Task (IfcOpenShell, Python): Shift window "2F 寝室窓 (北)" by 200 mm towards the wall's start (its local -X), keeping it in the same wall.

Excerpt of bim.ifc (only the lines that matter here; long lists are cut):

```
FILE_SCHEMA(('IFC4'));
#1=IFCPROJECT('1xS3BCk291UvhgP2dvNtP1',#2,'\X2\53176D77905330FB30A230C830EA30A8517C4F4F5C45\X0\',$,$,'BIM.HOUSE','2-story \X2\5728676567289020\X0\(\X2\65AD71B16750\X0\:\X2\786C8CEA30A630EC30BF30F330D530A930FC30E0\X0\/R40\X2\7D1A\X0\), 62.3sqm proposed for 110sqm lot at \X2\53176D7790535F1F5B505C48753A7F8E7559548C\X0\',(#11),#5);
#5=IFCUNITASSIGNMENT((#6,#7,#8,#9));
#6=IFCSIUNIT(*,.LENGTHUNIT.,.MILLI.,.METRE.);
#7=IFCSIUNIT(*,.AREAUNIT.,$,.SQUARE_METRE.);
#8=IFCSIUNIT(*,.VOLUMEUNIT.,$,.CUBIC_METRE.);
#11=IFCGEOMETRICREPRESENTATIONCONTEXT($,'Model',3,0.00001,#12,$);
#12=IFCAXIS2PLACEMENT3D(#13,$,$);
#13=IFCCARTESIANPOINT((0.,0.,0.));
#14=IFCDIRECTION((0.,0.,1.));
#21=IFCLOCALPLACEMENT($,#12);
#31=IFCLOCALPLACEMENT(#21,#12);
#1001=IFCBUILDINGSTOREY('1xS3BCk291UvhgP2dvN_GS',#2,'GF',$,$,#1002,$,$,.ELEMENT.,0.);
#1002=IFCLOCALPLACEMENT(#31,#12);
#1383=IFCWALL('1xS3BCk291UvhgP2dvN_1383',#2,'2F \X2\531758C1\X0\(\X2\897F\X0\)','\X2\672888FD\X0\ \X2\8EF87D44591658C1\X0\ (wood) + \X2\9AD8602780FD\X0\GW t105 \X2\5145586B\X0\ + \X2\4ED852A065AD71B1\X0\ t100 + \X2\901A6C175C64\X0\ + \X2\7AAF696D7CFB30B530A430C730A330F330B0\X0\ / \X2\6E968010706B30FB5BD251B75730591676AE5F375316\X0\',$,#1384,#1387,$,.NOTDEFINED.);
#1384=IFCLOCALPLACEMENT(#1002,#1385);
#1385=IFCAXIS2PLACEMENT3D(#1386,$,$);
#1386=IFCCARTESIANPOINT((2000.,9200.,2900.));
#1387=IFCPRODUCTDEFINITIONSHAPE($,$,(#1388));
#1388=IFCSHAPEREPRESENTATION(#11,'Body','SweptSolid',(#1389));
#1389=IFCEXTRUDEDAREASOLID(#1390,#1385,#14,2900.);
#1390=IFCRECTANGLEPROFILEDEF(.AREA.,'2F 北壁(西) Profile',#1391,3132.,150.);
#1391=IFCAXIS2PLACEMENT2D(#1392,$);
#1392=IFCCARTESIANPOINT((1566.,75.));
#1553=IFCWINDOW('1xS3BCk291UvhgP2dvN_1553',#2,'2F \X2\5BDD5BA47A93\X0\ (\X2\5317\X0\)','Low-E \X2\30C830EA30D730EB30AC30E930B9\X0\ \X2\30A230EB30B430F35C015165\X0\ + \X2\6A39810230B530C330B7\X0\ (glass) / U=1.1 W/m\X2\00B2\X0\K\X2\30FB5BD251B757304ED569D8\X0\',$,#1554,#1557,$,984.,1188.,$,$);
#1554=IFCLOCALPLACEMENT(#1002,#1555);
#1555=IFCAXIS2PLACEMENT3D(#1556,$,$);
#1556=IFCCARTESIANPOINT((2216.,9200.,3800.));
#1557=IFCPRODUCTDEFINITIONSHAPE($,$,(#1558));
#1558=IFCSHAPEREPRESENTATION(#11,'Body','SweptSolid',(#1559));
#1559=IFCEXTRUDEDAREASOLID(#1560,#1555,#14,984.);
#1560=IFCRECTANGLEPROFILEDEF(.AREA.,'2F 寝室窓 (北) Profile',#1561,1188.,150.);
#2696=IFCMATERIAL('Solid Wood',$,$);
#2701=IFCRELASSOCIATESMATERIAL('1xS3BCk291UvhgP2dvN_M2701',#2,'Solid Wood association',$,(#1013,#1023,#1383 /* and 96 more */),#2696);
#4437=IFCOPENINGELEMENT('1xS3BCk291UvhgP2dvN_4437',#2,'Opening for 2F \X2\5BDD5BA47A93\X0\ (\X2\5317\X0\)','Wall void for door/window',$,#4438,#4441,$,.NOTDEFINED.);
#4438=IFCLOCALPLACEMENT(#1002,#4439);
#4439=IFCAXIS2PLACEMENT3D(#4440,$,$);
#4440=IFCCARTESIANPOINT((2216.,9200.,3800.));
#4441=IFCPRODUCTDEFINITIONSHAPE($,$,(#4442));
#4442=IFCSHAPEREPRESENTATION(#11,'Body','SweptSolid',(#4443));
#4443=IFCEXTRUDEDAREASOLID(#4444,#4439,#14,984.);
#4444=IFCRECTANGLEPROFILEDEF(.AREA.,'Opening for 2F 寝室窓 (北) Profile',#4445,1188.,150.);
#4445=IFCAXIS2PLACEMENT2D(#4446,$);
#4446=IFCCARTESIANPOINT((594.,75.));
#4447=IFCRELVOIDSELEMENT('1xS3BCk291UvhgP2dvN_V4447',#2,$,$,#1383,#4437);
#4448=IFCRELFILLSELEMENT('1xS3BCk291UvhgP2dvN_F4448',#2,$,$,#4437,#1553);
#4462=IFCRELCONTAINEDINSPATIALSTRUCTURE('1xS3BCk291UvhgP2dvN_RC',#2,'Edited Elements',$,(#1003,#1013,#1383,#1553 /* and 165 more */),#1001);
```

```python
import ifcopenshell
import ifcopenshell.api.geometry
import ifcopenshell.util.placement
import ifcopenshell.util.unit

model = ifcopenshell.open("bim.ifc")
unit_scale = ifcopenshell.util.unit.calculate_unit_scale(model)

window = model.by_guid("1xS3BCk291UvhgP2dvN_1553")
opening = window.FillsVoids[0].RelatingOpeningElement
wall = opening.VoidsElements[0].RelatingBuildingElement

wall_matrix = ifcopenshell.util.placement.get_local_placement(wall.ObjectPlacement)
shift = wall_matrix[:3, 0] * -0.2 / unit_scale
before = ifcopenshell.util.placement.get_local_placement(window.ObjectPlacement)[:3, 3].copy()

# The window is not placed relative to its opening, so move both.
for product in (opening, window):
    matrix = ifcopenshell.util.placement.get_local_placement(product.ObjectPlacement)
    matrix[:3, 3] += shift
    ifcopenshell.api.geometry.edit_object_placement(model, product=product, matrix=matrix, is_si=False)

after = ifcopenshell.util.placement.get_local_placement(window.ObjectPlacement)[:3, 3]
print("window moved by", (after - before).round(3) + 0.0)

model.write("bim_updated.ifc")
```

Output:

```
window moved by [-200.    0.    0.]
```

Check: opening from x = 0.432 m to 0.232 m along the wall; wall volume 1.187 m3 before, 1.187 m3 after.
